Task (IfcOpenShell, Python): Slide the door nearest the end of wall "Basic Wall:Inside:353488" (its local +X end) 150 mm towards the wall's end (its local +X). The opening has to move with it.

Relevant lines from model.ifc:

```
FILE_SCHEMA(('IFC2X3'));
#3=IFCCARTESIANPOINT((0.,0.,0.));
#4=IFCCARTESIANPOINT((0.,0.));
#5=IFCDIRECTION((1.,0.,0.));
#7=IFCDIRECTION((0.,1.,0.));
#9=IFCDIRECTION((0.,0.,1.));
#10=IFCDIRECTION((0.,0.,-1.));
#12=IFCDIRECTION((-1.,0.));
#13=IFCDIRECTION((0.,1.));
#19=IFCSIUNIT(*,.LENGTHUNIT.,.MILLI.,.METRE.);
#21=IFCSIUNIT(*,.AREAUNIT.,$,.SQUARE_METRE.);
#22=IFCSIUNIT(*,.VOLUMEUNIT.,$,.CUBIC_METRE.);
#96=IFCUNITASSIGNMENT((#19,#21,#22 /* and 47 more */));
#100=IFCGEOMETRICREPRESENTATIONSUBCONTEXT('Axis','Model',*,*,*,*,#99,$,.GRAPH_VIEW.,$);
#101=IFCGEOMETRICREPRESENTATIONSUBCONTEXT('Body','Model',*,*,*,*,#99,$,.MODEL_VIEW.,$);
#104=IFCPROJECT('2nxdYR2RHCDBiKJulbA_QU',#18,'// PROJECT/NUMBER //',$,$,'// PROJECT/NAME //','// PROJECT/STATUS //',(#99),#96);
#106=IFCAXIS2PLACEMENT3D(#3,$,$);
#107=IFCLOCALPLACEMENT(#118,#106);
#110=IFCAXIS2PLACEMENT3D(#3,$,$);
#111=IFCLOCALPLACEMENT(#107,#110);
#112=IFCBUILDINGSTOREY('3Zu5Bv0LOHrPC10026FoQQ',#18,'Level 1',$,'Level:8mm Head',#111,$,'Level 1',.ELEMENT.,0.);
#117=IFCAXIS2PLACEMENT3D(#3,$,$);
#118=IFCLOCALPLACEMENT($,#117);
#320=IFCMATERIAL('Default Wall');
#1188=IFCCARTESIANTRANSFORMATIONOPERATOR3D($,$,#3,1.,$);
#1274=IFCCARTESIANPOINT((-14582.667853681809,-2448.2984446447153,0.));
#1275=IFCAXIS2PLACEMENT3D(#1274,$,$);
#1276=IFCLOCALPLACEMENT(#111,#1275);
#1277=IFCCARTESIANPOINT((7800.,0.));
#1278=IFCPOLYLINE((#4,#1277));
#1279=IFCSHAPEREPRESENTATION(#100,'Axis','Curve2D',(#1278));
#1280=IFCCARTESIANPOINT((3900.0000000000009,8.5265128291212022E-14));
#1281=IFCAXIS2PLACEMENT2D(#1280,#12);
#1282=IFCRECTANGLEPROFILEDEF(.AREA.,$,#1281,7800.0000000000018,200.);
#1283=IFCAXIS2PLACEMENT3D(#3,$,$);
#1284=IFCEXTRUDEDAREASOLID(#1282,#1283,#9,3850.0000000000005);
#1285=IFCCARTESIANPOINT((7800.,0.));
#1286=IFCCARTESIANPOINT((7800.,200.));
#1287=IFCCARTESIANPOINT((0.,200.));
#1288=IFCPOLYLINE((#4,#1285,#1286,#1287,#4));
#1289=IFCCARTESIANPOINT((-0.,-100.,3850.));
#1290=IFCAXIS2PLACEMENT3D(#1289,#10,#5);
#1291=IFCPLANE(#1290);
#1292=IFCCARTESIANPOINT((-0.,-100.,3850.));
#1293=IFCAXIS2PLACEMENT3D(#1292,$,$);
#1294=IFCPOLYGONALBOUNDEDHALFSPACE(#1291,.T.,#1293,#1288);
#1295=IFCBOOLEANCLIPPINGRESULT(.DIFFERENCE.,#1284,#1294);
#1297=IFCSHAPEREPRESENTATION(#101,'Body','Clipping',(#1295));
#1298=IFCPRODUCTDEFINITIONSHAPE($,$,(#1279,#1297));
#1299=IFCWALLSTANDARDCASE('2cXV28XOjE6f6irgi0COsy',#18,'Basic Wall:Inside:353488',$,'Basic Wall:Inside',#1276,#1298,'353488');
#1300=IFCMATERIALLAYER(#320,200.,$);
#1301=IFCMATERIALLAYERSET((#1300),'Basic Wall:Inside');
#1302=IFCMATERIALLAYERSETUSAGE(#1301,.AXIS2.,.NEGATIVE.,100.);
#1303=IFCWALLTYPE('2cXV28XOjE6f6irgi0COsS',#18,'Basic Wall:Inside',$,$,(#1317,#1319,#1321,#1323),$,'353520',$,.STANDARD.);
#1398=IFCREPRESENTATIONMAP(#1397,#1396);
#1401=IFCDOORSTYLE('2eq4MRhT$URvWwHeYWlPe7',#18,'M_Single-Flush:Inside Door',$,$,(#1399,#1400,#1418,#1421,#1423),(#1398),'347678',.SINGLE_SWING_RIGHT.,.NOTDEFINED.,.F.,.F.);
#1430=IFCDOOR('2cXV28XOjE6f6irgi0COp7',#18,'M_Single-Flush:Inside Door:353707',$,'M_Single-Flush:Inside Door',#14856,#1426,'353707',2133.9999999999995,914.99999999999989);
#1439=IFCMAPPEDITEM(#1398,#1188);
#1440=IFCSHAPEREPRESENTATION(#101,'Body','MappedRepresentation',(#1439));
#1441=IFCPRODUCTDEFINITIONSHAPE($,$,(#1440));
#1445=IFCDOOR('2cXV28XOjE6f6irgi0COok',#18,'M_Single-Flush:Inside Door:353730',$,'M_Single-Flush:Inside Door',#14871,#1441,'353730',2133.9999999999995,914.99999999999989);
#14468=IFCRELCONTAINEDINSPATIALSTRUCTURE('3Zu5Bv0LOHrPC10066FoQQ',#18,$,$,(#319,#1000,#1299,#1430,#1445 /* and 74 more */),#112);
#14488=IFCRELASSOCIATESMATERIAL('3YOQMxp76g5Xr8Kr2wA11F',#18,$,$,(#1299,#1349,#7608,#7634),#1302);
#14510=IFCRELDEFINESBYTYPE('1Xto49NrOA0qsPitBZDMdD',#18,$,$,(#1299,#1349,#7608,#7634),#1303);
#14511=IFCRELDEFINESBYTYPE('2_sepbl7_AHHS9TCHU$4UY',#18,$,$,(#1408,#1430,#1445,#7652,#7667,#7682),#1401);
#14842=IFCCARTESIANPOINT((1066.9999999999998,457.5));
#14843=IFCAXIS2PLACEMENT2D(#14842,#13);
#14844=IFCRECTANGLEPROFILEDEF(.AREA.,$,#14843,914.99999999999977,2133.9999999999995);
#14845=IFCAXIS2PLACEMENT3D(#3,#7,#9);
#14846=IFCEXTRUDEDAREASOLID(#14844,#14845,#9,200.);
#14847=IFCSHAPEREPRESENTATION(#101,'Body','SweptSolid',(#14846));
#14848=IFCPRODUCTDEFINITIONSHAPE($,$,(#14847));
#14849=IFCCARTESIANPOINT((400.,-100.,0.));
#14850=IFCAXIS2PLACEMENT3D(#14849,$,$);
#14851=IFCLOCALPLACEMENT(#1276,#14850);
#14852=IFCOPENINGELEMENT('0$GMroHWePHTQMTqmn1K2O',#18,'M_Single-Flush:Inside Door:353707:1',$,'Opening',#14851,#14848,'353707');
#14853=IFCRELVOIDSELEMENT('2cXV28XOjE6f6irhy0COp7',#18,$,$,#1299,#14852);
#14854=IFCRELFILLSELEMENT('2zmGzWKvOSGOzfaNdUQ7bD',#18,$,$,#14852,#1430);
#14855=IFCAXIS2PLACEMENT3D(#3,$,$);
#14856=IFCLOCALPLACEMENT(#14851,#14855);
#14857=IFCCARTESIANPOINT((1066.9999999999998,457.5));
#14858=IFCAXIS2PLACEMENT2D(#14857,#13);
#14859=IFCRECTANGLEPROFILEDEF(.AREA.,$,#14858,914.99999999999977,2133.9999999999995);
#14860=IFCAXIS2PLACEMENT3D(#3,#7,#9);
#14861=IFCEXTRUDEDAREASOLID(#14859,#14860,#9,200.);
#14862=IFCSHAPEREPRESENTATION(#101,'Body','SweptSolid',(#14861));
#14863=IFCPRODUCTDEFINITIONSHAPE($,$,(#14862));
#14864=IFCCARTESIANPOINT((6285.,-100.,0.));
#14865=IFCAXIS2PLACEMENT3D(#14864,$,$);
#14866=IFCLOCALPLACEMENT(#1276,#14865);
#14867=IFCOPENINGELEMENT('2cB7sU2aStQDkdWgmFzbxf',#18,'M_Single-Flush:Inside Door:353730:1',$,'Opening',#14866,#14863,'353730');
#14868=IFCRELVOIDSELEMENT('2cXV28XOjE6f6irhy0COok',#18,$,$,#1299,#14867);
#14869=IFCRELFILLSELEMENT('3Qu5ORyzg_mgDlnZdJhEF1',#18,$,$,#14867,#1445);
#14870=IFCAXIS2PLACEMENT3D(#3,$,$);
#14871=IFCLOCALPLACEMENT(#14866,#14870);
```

```python
import ifcopenshell
import ifcopenshell.api.geometry
import ifcopenshell.util.placement
import ifcopenshell.util.unit

model = ifcopenshell.open("model.ifc")
unit_scale = ifcopenshell.util.unit.calculate_unit_scale(model)

door = model.by_guid("2cXV28XOjE6f6irgi0COok")
opening = door.FillsVoids[0].RelatingOpeningElement
wall = opening.VoidsElements[0].RelatingBuildingElement

wall_matrix = ifcopenshell.util.placement.get_local_placement(wall.ObjectPlacement)
shift = wall_matrix[:3, 0] * 0.15 / unit_scale
before = ifcopenshell.util.placement.get_local_placement(door.ObjectPlacement)[:3, 3].copy()

# The door is placed relative to its opening, so it follows when the opening moves.
matrix = ifcopenshell.util.placement.get_local_placement(opening.ObjectPlacement)
matrix[:3, 3] += shift
ifcopenshell.api.geometry.edit_object_placement(
    model, product=opening, matrix=matrix, is_si=False, should_transform_children=True
)

after = ifcopenshell.util.placement.get_local_placement(door.ObjectPlacement)[:3, 3]
print("door moved by", (after - before).round(3) + 0.0)

model.write("model_v2.ifc")
```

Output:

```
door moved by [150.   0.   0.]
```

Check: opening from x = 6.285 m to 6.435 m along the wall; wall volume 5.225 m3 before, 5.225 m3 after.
